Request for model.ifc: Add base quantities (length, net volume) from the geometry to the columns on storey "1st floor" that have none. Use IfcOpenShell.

First a look at what the model holds.

```python
import ifcopenshell
import ifcopenshell.util.element
import ifcopenshell.util.unit

model = ifcopenshell.open("model.ifc")
print(model.schema)
for unit_type in ("LENGTHUNIT", "AREAUNIT", "VOLUMEUNIT"):
    print(unit_type, ifcopenshell.util.unit.calculate_unit_scale(model, unit_type))
storey = next(s for s in model.by_type("IfcBuildingStorey") if s.Name == "1st floor")
columns = [e for e in ifcopenshell.util.element.get_decomposition(storey) if e.is_a("IfcColumn")]
for e in sorted(columns, key=lambda e: e.id()):
    print(e.id(), e.is_a(), e.Name, list(ifcopenshell.util.element.get_psets(e, qtos_only=True)), sep=" | ")
```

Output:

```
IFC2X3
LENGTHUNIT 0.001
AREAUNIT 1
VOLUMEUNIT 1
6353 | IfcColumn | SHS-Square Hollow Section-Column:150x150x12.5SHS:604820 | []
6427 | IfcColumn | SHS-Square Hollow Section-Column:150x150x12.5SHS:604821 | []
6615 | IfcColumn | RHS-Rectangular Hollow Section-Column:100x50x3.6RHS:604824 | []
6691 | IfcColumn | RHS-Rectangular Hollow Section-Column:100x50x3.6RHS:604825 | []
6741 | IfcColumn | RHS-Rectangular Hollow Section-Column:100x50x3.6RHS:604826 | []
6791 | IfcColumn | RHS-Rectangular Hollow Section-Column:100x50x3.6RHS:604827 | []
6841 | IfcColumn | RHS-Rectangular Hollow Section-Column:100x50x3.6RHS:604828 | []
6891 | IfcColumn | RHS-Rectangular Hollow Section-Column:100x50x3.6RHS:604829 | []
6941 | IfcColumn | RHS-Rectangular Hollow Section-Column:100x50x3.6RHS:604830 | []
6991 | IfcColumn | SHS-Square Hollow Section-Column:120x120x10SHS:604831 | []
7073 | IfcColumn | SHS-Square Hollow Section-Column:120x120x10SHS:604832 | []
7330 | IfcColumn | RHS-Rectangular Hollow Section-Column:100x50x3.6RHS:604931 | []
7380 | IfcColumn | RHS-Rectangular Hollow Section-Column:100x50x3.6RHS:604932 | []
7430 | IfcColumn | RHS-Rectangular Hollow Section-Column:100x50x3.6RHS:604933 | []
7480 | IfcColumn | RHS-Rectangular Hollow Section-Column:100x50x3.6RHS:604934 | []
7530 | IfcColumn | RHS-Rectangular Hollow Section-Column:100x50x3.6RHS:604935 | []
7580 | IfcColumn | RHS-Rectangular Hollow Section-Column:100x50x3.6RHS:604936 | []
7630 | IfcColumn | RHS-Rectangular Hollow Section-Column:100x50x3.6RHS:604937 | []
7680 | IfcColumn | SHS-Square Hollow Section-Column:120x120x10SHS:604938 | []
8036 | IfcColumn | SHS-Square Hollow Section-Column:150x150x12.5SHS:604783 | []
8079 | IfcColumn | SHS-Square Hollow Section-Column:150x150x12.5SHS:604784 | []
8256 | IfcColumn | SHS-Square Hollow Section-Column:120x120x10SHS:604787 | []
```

```python
import ifcopenshell
import ifcopenshell.api.pset
import ifcopenshell.geom
import ifcopenshell.util.element
import ifcopenshell.util.shape
import ifcopenshell.util.unit

model = ifcopenshell.open("model.ifc")
unit_scale = ifcopenshell.util.unit.calculate_unit_scale(model)
volume_scale = ifcopenshell.util.unit.calculate_unit_scale(model, "VOLUMEUNIT")
settings = ifcopenshell.geom.settings()

storey = next(s for s in model.by_type("IfcBuildingStorey") if s.Name == "1st floor")
columns = [e for e in ifcopenshell.util.element.get_decomposition(storey) if e.is_a("IfcColumn")]

for e in sorted(columns, key=lambda e: e.id()):
    if ifcopenshell.util.element.get_psets(e, qtos_only=True, should_inherit=False):
        continue
    # Geometry comes back in metres, in the element's own axes.
    shape = ifcopenshell.geom.create_shape(settings, e)
    values = {
        "Length": ifcopenshell.util.shape.get_z(shape.geometry) / unit_scale,
        "NetVolume": ifcopenshell.util.shape.get_volume(shape.geometry) / volume_scale,
    }
    qto = ifcopenshell.api.pset.add_qto(model, product=e, name="BaseQuantities")
    ifcopenshell.api.pset.edit_qto(model, qto=qto, properties=values)
    print(e.id(), {k: round(v, 3) for k, v in values.items()})

model.write("model_updated.ifc")
```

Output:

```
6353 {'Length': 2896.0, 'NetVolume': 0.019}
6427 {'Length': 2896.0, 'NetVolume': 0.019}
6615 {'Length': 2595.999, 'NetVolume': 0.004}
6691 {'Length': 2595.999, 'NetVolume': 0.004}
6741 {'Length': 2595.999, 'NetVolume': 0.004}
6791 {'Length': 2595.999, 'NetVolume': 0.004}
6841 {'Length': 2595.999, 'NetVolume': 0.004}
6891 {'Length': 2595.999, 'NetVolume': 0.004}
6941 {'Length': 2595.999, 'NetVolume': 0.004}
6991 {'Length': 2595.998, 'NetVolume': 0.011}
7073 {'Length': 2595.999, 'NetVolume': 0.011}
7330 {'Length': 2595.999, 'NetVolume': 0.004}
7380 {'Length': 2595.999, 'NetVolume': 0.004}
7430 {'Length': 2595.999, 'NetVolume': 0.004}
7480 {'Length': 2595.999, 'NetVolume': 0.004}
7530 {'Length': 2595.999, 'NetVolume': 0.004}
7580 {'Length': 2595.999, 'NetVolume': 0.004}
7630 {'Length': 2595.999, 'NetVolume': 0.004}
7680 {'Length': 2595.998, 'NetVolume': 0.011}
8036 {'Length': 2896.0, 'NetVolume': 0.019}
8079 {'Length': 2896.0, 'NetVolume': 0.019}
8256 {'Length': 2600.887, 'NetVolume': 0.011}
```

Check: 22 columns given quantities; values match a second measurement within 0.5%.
